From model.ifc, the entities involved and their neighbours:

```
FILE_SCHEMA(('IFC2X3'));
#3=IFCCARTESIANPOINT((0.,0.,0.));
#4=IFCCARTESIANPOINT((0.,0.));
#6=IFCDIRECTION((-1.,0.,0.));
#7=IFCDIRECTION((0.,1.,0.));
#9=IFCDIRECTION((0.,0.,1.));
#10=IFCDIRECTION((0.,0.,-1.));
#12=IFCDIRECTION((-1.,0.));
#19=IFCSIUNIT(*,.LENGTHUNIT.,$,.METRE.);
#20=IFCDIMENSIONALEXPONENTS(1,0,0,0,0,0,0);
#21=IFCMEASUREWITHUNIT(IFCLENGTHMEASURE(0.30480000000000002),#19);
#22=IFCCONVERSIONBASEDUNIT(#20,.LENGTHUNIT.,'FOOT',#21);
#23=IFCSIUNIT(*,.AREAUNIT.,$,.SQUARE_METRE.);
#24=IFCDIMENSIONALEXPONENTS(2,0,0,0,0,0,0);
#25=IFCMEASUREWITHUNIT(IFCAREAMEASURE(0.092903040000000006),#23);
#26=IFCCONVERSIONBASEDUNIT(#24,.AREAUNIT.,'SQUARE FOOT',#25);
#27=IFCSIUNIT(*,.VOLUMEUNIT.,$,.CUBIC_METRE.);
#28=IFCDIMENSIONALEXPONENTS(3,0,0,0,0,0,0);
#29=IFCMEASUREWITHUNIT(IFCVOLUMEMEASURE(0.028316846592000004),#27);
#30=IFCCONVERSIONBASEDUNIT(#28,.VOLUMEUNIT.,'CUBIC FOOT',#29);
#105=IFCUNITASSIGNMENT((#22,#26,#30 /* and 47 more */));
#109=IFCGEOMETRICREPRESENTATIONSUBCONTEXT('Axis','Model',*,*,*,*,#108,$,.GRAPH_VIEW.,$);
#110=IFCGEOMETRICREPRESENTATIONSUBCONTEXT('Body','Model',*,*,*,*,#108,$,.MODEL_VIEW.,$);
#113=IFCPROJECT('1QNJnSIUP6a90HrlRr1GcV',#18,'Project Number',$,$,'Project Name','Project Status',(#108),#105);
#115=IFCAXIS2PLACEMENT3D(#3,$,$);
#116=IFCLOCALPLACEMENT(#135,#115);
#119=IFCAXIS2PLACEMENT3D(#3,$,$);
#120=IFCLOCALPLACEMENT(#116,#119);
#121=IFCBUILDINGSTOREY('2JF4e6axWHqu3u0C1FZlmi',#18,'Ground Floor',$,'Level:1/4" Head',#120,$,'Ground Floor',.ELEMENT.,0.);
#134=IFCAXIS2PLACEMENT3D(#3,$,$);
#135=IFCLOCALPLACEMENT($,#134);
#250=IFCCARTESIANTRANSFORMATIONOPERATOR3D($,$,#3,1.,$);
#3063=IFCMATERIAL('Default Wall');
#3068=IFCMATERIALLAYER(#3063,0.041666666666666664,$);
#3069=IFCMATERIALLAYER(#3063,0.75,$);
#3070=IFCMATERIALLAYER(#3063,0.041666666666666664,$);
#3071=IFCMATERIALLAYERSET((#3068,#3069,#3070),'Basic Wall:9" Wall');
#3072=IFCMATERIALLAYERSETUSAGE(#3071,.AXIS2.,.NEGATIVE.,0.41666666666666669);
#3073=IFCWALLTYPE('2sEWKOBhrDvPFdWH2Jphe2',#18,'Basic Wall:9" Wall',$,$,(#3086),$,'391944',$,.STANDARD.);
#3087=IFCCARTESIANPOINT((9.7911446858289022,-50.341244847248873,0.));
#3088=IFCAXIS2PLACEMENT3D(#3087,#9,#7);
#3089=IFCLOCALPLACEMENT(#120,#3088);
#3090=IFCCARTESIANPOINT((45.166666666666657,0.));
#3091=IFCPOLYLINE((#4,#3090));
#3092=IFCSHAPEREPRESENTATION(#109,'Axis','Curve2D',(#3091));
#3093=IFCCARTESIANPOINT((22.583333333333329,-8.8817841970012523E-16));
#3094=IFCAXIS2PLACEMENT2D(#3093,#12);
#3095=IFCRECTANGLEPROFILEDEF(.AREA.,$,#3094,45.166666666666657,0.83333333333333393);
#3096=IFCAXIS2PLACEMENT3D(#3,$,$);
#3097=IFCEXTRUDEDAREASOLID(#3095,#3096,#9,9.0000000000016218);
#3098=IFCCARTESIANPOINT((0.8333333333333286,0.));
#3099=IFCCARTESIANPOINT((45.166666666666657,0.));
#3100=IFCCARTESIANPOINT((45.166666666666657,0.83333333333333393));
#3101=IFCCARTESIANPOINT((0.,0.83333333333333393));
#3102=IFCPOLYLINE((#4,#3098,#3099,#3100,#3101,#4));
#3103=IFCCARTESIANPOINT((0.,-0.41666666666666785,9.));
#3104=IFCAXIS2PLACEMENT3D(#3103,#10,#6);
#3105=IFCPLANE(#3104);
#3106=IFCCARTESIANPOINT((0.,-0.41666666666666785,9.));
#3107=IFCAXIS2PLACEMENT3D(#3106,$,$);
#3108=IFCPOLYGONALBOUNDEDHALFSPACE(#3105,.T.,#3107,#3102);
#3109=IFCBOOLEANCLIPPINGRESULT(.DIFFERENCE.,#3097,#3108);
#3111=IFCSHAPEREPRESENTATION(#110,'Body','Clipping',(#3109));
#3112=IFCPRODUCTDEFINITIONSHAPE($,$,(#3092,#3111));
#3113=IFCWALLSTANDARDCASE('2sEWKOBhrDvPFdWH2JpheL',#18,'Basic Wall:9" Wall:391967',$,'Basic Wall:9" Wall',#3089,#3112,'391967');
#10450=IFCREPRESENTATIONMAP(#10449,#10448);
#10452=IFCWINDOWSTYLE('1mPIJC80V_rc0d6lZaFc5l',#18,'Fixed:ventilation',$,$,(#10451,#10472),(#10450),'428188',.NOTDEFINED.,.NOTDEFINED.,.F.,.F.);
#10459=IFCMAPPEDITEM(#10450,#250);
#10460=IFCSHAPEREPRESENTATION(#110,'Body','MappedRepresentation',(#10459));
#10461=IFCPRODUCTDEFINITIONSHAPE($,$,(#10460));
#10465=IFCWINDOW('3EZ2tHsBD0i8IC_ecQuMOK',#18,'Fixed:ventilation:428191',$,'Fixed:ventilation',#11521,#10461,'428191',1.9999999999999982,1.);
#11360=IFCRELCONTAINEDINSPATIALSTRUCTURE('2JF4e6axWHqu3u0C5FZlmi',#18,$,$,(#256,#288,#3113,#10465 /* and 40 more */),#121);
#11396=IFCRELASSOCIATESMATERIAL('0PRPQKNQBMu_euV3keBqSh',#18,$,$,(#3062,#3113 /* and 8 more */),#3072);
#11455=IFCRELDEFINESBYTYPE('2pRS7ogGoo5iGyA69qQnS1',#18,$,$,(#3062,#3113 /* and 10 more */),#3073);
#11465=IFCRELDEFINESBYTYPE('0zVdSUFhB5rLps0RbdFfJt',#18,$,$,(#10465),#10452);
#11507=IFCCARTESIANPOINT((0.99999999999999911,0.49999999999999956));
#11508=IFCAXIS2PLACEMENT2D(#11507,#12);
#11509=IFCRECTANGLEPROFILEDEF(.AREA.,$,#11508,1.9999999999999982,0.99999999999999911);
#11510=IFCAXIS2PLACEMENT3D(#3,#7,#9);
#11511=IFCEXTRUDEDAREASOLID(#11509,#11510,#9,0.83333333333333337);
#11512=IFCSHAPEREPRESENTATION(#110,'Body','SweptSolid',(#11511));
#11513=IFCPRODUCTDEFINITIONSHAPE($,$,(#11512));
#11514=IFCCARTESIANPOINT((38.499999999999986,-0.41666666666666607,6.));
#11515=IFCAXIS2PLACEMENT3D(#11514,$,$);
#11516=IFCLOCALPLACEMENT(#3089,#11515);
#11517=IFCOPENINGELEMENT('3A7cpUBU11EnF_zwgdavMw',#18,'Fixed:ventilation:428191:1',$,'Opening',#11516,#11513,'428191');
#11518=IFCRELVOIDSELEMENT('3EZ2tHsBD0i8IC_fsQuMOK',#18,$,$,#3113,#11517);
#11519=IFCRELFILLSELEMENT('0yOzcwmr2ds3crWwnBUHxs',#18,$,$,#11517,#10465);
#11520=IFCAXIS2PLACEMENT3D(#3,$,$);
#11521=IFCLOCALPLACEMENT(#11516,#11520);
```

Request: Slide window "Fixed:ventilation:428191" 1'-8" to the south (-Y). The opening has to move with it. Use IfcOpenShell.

```python
import ifcopenshell
import ifcopenshell.api.geometry
import ifcopenshell.util.placement
import ifcopenshell.util.unit

model = ifcopenshell.open("model.ifc")
unit_scale = ifcopenshell.util.unit.calculate_unit_scale(model)

window = model.by_guid("3EZ2tHsBD0i8IC_ecQuMOK")
opening = window.FillsVoids[0].RelatingOpeningElement
wall = opening.VoidsElements[0].RelatingBuildingElement

wall_matrix = ifcopenshell.util.placement.get_local_placement(wall.ObjectPlacement)
shift = wall_matrix[:3, 0] * -20 * 0.0254 / unit_scale
before = ifcopenshell.util.placement.get_local_placement(window.ObjectPlacement)[:3, 3].copy()

# The window is placed relative to its opening, so it follows when the opening moves.
matrix = ifcopenshell.util.placement.get_local_placement(opening.ObjectPlacement)
matrix[:3, 3] += shift
ifcopenshell.api.geometry.edit_object_placement(
    model, product=opening, matrix=matrix, is_si=False, should_transform_children=True
)

after = ifcopenshell.util.placement.get_local_placement(window.ObjectPlacement)[:3, 3]
print("window moved by", (after - before).round(3) + 0.0)

model.write("model_rev.ifc")
```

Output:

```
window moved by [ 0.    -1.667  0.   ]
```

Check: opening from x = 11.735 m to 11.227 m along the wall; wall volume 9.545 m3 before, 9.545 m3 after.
